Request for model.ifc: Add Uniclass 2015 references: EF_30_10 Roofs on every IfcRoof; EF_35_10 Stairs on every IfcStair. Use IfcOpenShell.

First a look at what the model holds.

```python
import ifcopenshell

model = ifcopenshell.open("model.ifc")
print(model.schema)
print("classifications:", [c.Name for c in model.by_type("IfcClassification")])
for ifc_class in ("IfcDoor", "IfcRoof", "IfcStair", "IfcWall", "IfcWindow"):
    print(ifc_class, len(model.by_type(ifc_class)))
```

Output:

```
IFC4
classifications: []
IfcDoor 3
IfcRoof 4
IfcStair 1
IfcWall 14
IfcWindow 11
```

```python
import ifcopenshell
import ifcopenshell.api.classification

model = ifcopenshell.open("model.ifc")

system = ifcopenshell.api.classification.add_classification(model, classification="Uniclass 2015")

codes = {
    "IfcRoof": ("EF_30_10", "Roofs"),
    "IfcStair": ("EF_35_10", "Stairs"),
}
for ifc_class, (code, name) in codes.items():
    products = model.by_type(ifc_class)
    ifcopenshell.api.classification.add_reference(
        model, products=products, classification=system, identification=code, name=name
    )
    print(code, len(products))

model.write("model_v2.ifc")
```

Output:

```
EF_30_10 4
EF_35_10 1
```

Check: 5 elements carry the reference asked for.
